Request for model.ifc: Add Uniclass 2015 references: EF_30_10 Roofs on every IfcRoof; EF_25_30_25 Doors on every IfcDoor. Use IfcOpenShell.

First a look at what the model holds.

```python
import ifcopenshell

model = ifcopenshell.open("model.ifc")
print(model.schema)
print("classifications:", [c.Name for c in model.by_type("IfcClassification")])
for ifc_class in ("IfcDoor", "IfcRoof", "IfcStair", "IfcWall", "IfcWindow"):
    print(ifc_class, len(model.by_type(ifc_class)))
```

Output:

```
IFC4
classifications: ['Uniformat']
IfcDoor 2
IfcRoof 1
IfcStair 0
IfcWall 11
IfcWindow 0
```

```python
import ifcopenshell
import ifcopenshell.api.classification

model = ifcopenshell.open("model.ifc")

system = ifcopenshell.api.classification.add_classification(model, classification="Uniclass 2015")

codes = {
    "IfcRoof": ("EF_30_10", "Roofs"),
    "IfcDoor": ("EF_25_30_25", "Doors"),
}
for ifc_class, (code, name) in codes.items():
    products = model.by_type(ifc_class)
    ifcopenshell.api.classification.add_reference(
        model, products=products, classification=system, identification=code, name=name
    )
    print(code, len(products))

model.write("model_updated.ifc")
```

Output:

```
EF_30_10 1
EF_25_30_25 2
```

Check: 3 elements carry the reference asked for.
